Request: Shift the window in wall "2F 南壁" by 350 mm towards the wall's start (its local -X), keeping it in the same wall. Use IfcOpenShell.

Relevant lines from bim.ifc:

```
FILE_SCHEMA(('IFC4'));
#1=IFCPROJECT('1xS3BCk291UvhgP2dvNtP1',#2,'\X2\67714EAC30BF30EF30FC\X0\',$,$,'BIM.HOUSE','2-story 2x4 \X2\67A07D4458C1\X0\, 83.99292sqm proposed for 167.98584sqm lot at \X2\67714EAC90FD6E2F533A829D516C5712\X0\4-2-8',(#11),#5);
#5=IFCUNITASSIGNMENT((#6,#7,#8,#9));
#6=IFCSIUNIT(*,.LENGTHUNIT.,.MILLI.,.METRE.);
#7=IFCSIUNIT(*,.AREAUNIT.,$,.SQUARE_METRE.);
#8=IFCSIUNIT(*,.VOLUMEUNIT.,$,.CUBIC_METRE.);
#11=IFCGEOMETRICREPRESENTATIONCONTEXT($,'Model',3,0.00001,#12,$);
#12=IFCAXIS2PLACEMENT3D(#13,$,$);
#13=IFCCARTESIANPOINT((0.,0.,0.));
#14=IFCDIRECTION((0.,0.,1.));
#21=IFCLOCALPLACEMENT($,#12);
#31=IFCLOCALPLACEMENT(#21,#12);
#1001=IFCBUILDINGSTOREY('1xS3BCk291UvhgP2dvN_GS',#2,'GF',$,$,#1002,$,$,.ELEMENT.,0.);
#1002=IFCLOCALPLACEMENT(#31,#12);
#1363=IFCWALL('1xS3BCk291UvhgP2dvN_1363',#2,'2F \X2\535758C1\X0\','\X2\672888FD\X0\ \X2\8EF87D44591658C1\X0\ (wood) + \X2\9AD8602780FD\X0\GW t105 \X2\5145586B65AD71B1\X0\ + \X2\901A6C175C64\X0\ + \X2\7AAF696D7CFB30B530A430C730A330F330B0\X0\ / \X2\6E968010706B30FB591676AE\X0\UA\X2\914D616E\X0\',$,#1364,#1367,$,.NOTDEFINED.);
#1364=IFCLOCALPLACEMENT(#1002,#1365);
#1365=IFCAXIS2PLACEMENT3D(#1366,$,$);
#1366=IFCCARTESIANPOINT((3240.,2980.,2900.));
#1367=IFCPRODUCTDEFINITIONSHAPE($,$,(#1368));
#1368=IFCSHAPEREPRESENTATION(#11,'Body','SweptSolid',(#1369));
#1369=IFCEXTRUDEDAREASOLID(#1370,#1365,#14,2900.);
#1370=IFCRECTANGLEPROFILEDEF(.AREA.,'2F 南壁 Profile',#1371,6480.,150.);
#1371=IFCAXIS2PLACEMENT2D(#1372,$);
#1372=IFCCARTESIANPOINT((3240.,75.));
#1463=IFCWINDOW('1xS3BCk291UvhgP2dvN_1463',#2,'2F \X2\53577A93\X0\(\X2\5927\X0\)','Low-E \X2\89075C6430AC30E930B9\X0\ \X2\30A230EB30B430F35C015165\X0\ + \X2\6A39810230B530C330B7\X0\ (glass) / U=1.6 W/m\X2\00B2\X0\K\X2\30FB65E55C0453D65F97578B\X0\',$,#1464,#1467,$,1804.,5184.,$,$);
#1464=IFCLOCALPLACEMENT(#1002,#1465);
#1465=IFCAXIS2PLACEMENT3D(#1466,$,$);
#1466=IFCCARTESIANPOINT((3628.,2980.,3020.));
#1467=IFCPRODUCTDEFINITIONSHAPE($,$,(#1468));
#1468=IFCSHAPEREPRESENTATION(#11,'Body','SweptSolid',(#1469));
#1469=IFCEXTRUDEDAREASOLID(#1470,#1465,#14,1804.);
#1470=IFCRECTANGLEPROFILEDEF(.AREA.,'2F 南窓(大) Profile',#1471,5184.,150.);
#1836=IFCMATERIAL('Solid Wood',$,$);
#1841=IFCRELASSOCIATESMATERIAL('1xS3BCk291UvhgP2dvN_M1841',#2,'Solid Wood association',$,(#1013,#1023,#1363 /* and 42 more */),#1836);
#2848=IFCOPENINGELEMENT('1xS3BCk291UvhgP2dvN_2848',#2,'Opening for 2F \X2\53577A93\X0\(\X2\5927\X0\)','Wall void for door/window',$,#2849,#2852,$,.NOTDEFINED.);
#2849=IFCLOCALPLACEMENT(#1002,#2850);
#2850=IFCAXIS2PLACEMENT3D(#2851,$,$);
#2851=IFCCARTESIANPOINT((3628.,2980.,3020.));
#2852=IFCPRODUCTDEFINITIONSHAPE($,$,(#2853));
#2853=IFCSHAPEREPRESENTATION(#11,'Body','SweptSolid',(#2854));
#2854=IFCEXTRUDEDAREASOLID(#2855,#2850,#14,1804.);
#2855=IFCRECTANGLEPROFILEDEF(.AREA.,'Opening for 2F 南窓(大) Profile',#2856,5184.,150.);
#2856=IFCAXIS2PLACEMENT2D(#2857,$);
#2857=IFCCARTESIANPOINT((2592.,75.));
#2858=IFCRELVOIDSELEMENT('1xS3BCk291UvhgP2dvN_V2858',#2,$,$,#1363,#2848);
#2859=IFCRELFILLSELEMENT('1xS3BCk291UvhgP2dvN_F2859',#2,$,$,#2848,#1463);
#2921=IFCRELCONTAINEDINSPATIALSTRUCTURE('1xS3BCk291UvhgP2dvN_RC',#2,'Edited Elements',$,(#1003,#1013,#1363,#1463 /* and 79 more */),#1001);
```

```python
import ifcopenshell
import ifcopenshell.api.geometry
import ifcopenshell.util.placement
import ifcopenshell.util.unit

model = ifcopenshell.open("bim.ifc")
unit_scale = ifcopenshell.util.unit.calculate_unit_scale(model)

window = model.by_guid("1xS3BCk291UvhgP2dvN_1463")
opening = window.FillsVoids[0].RelatingOpeningElement
wall = opening.VoidsElements[0].RelatingBuildingElement

wall_matrix = ifcopenshell.util.placement.get_local_placement(wall.ObjectPlacement)
shift = wall_matrix[:3, 0] * -0.35 / unit_scale
before = ifcopenshell.util.placement.get_local_placement(window.ObjectPlacement)[:3, 3].copy()

# The window is not placed relative to its opening, so move both.
for product in (opening, window):
    matrix = ifcopenshell.util.placement.get_local_placement(product.ObjectPlacement)
    matrix[:3, 3] += shift
    ifcopenshell.api.geometry.edit_object_placement(model, product=product, matrix=matrix, is_si=False)

after = ifcopenshell.util.placement.get_local_placement(window.ObjectPlacement)[:3, 3]
print("window moved by", (after - before).round(3) + 0.0)

model.write("bim_rev.ifc")
```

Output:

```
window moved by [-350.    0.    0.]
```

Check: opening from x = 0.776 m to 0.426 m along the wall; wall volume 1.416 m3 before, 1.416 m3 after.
